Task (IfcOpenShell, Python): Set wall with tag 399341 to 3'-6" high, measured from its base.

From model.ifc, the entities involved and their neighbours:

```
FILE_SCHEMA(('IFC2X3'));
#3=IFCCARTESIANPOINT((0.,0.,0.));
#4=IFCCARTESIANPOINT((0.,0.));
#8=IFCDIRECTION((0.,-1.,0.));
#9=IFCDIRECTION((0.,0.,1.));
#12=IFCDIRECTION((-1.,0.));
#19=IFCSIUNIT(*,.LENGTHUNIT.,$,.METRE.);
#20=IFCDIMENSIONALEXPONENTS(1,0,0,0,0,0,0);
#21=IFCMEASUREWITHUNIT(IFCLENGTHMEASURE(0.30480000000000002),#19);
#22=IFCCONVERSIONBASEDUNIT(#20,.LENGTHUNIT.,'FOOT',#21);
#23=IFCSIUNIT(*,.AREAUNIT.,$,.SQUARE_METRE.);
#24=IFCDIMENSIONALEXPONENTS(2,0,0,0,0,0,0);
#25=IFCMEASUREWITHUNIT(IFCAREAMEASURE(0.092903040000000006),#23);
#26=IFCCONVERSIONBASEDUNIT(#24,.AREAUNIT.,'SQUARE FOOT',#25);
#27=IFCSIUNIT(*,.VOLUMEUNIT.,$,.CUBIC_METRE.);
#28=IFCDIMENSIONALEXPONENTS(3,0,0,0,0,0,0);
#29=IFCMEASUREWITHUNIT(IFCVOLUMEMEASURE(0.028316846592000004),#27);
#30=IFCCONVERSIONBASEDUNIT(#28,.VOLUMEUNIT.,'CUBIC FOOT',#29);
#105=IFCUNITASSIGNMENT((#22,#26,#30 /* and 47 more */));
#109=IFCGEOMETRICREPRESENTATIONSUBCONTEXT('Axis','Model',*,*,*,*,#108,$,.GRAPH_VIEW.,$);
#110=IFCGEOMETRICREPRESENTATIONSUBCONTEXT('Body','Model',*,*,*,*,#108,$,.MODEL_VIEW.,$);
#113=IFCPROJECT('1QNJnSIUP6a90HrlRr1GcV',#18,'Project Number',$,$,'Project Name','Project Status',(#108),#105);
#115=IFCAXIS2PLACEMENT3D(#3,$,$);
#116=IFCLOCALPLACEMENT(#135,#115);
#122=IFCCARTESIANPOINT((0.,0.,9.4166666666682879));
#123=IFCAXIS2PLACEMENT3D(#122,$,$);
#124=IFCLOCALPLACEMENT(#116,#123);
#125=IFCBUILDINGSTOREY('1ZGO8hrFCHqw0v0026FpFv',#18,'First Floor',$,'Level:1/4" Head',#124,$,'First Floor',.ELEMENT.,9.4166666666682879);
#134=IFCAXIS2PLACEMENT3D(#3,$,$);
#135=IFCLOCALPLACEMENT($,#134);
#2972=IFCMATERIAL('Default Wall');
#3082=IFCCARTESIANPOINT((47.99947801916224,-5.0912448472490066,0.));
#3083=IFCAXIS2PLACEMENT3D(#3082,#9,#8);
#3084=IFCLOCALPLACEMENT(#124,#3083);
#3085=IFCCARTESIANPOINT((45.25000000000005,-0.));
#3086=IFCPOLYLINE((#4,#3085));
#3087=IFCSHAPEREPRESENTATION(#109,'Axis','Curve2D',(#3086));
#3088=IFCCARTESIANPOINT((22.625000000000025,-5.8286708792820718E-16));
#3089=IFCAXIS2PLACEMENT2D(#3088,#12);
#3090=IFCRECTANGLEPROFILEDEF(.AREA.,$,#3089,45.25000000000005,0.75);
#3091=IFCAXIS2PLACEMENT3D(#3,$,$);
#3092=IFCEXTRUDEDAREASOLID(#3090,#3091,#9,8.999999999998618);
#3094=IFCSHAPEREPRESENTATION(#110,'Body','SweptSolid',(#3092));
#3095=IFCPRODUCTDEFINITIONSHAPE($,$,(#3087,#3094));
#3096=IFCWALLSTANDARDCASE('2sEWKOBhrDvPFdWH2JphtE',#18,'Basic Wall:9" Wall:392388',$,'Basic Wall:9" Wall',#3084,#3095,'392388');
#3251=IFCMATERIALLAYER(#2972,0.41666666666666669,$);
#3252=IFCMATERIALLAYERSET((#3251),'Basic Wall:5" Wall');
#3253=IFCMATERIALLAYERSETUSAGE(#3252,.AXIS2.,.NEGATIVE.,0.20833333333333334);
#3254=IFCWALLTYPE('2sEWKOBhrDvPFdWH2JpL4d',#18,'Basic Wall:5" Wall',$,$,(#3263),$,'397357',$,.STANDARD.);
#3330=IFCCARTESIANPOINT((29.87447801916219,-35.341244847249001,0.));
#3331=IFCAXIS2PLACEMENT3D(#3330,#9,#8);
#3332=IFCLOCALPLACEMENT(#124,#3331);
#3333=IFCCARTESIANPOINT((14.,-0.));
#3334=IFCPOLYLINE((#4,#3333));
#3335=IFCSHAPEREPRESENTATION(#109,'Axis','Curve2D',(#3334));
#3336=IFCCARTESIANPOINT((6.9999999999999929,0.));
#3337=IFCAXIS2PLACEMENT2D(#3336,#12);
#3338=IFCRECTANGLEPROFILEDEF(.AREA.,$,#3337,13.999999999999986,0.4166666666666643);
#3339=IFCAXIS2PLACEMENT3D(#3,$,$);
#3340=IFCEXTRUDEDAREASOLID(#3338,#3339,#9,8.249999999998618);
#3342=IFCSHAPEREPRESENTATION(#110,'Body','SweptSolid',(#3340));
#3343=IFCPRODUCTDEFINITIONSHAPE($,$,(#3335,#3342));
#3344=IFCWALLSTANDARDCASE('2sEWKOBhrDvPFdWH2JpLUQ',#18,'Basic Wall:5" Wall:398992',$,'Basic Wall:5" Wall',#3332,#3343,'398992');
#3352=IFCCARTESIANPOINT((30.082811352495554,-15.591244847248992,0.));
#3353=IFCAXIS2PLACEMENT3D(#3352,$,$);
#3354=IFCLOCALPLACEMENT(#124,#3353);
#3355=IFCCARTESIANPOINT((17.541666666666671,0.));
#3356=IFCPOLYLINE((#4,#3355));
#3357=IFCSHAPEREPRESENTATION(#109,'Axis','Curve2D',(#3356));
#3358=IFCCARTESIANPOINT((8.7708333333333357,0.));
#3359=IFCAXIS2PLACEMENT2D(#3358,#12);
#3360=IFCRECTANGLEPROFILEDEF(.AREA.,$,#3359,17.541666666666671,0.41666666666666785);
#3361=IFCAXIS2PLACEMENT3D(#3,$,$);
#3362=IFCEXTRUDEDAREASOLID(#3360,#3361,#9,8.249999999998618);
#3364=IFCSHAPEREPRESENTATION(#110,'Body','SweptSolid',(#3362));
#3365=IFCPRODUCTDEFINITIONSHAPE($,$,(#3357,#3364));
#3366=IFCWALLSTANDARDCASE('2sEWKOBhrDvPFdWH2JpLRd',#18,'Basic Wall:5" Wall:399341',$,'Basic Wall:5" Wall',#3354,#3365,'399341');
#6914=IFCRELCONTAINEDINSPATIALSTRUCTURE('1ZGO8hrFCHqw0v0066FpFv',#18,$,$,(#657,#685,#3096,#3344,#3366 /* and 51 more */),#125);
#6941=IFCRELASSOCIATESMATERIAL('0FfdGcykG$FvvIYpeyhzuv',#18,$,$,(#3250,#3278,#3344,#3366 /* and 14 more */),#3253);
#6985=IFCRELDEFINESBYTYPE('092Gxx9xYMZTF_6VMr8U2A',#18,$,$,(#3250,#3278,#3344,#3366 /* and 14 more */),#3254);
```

```python
import ifcopenshell
import ifcopenshell.geom
import ifcopenshell.util.representation
import ifcopenshell.util.shape
import ifcopenshell.util.unit

model = ifcopenshell.open("model.ifc")
unit_scale = ifcopenshell.util.unit.calculate_unit_scale(model)
settings = ifcopenshell.geom.settings()


def volume(element):
    """Net volume in cubic metres, openings subtracted."""
    shape = ifcopenshell.geom.create_shape(settings, element)
    return ifcopenshell.util.shape.get_volume(shape.geometry)


wall = model.by_id(3366)
before = volume(wall)

body = ifcopenshell.util.representation.get_representation(wall, "Model", "Body")
solid = body.Items[0]
old_height = solid.Depth
solid.Depth = 42 * 0.0254 / unit_scale
after = volume(wall)

print(f"height {old_height:g} -> {solid.Depth:g}, volume {before:.3f} -> {after:.3f} m3")

model.write("model_v2.ifc")
```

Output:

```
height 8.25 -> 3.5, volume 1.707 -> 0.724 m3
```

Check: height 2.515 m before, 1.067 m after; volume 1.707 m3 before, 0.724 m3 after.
